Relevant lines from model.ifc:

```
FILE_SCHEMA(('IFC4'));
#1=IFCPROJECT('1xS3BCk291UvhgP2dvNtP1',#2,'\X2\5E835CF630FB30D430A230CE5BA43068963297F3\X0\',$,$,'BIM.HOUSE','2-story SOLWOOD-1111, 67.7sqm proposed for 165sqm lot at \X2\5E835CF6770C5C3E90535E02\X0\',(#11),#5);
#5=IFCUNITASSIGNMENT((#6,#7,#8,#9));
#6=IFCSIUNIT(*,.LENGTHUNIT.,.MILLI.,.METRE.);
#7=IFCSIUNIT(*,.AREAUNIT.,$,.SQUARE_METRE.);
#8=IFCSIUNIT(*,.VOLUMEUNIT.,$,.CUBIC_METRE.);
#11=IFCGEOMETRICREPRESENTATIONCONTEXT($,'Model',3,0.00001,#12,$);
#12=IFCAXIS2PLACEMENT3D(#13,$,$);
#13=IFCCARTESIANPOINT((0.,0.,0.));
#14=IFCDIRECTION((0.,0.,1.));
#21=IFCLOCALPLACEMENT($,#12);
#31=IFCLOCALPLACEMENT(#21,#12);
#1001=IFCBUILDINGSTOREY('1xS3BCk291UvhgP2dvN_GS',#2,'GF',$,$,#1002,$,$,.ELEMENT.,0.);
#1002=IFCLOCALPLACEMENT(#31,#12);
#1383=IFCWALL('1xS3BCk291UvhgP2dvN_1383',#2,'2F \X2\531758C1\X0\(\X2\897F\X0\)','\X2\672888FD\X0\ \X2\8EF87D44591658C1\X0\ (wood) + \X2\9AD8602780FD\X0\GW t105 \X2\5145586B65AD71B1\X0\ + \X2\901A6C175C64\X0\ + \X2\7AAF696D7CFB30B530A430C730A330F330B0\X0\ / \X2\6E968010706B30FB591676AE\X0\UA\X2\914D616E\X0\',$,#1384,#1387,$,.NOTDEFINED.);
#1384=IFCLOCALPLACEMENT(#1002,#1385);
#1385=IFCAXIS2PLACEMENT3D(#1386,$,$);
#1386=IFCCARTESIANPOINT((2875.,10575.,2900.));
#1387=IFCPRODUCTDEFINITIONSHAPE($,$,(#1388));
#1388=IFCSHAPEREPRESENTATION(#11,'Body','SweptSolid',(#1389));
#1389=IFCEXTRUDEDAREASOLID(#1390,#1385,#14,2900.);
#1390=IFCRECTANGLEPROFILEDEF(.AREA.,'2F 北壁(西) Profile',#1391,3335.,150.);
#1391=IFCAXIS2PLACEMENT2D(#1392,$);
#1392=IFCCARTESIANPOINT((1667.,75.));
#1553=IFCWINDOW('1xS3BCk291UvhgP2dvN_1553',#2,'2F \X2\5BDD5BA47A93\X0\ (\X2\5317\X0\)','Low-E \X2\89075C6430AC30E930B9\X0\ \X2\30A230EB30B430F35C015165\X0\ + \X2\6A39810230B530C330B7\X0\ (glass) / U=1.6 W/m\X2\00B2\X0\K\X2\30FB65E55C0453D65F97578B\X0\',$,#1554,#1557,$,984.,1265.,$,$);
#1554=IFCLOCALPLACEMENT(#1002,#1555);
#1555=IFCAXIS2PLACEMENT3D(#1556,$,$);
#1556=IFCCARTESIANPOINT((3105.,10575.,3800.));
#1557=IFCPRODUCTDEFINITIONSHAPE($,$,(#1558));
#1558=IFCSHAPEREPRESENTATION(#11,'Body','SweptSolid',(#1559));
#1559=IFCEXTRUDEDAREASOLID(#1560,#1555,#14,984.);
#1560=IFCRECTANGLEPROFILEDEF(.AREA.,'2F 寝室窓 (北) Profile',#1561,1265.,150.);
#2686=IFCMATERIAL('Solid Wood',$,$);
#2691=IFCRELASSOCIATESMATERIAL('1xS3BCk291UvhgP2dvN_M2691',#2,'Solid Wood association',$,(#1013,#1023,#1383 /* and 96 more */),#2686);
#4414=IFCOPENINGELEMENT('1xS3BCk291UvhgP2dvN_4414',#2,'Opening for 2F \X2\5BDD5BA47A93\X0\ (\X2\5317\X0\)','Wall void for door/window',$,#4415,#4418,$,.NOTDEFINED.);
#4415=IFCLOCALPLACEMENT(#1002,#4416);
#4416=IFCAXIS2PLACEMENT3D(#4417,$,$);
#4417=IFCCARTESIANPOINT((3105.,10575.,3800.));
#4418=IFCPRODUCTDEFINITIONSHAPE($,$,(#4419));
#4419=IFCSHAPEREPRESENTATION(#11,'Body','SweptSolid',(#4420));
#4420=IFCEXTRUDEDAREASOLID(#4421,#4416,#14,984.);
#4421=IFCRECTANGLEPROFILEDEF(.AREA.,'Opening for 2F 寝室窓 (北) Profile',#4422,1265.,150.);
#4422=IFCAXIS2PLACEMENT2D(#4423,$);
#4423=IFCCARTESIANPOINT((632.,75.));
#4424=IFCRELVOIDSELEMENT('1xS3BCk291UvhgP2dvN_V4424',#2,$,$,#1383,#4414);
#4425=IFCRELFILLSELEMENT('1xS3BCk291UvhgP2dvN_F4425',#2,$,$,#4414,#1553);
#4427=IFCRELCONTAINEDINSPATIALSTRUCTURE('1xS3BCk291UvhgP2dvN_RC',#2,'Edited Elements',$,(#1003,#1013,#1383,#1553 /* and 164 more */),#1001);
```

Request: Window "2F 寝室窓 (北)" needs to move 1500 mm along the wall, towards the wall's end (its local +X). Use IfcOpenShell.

```python
import ifcopenshell
import ifcopenshell.api.geometry
import ifcopenshell.util.placement

model = ifcopenshell.open("model.ifc")

window = model.by_guid("1xS3BCk291UvhgP2dvN_1553")
opening = window.FillsVoids[0].RelatingOpeningElement
wall = opening.VoidsElements[0].RelatingBuildingElement

wall_matrix = ifcopenshell.util.placement.get_local_placement(wall.ObjectPlacement)
shift = wall_matrix[:3, 0] * 1500.0
before = ifcopenshell.util.placement.get_local_placement(window.ObjectPlacement)[:3, 3].copy()

# The window is not placed relative to its opening, so move both.
for product in (opening, window):
    matrix = ifcopenshell.util.placement.get_local_placement(product.ObjectPlacement)
    matrix[:3, 3] += shift
    ifcopenshell.api.geometry.edit_object_placement(model, product=product, matrix=matrix, is_si=False)

after = ifcopenshell.util.placement.get_local_placement(window.ObjectPlacement)[:3, 3]
print("window moved by", (after - before).round(3) + 0.0)

model.write("model_updated.ifc")
```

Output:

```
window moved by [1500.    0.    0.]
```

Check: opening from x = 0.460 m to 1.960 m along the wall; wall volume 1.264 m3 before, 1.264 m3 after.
